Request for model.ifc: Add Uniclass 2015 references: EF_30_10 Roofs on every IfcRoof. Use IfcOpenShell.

First a look at what the model holds.

```python
import ifcopenshell

model = ifcopenshell.open("model.ifc")
print(model.schema)
print("classifications:", [c.Name for c in model.by_type("IfcClassification")])
for ifc_class in ("IfcDoor", "IfcRoof", "IfcStair", "IfcWall", "IfcWindow"):
    print(ifc_class, len(model.by_type(ifc_class)))
```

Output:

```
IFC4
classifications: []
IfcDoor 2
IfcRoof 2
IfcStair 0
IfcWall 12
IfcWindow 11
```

```python
import ifcopenshell
import ifcopenshell.api.classification

model = ifcopenshell.open("model.ifc")

system = ifcopenshell.api.classification.add_classification(model, classification="Uniclass 2015")

codes = {
    "IfcRoof": ("EF_30_10", "Roofs"),
}
for ifc_class, (code, name) in codes.items():
    products = model.by_type(ifc_class)
    ifcopenshell.api.classification.add_reference(
        model, products=products, classification=system, identification=code, name=name
    )
    print(code, len(products))

model.write("model-out.ifc")
```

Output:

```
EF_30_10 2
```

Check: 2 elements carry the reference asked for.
